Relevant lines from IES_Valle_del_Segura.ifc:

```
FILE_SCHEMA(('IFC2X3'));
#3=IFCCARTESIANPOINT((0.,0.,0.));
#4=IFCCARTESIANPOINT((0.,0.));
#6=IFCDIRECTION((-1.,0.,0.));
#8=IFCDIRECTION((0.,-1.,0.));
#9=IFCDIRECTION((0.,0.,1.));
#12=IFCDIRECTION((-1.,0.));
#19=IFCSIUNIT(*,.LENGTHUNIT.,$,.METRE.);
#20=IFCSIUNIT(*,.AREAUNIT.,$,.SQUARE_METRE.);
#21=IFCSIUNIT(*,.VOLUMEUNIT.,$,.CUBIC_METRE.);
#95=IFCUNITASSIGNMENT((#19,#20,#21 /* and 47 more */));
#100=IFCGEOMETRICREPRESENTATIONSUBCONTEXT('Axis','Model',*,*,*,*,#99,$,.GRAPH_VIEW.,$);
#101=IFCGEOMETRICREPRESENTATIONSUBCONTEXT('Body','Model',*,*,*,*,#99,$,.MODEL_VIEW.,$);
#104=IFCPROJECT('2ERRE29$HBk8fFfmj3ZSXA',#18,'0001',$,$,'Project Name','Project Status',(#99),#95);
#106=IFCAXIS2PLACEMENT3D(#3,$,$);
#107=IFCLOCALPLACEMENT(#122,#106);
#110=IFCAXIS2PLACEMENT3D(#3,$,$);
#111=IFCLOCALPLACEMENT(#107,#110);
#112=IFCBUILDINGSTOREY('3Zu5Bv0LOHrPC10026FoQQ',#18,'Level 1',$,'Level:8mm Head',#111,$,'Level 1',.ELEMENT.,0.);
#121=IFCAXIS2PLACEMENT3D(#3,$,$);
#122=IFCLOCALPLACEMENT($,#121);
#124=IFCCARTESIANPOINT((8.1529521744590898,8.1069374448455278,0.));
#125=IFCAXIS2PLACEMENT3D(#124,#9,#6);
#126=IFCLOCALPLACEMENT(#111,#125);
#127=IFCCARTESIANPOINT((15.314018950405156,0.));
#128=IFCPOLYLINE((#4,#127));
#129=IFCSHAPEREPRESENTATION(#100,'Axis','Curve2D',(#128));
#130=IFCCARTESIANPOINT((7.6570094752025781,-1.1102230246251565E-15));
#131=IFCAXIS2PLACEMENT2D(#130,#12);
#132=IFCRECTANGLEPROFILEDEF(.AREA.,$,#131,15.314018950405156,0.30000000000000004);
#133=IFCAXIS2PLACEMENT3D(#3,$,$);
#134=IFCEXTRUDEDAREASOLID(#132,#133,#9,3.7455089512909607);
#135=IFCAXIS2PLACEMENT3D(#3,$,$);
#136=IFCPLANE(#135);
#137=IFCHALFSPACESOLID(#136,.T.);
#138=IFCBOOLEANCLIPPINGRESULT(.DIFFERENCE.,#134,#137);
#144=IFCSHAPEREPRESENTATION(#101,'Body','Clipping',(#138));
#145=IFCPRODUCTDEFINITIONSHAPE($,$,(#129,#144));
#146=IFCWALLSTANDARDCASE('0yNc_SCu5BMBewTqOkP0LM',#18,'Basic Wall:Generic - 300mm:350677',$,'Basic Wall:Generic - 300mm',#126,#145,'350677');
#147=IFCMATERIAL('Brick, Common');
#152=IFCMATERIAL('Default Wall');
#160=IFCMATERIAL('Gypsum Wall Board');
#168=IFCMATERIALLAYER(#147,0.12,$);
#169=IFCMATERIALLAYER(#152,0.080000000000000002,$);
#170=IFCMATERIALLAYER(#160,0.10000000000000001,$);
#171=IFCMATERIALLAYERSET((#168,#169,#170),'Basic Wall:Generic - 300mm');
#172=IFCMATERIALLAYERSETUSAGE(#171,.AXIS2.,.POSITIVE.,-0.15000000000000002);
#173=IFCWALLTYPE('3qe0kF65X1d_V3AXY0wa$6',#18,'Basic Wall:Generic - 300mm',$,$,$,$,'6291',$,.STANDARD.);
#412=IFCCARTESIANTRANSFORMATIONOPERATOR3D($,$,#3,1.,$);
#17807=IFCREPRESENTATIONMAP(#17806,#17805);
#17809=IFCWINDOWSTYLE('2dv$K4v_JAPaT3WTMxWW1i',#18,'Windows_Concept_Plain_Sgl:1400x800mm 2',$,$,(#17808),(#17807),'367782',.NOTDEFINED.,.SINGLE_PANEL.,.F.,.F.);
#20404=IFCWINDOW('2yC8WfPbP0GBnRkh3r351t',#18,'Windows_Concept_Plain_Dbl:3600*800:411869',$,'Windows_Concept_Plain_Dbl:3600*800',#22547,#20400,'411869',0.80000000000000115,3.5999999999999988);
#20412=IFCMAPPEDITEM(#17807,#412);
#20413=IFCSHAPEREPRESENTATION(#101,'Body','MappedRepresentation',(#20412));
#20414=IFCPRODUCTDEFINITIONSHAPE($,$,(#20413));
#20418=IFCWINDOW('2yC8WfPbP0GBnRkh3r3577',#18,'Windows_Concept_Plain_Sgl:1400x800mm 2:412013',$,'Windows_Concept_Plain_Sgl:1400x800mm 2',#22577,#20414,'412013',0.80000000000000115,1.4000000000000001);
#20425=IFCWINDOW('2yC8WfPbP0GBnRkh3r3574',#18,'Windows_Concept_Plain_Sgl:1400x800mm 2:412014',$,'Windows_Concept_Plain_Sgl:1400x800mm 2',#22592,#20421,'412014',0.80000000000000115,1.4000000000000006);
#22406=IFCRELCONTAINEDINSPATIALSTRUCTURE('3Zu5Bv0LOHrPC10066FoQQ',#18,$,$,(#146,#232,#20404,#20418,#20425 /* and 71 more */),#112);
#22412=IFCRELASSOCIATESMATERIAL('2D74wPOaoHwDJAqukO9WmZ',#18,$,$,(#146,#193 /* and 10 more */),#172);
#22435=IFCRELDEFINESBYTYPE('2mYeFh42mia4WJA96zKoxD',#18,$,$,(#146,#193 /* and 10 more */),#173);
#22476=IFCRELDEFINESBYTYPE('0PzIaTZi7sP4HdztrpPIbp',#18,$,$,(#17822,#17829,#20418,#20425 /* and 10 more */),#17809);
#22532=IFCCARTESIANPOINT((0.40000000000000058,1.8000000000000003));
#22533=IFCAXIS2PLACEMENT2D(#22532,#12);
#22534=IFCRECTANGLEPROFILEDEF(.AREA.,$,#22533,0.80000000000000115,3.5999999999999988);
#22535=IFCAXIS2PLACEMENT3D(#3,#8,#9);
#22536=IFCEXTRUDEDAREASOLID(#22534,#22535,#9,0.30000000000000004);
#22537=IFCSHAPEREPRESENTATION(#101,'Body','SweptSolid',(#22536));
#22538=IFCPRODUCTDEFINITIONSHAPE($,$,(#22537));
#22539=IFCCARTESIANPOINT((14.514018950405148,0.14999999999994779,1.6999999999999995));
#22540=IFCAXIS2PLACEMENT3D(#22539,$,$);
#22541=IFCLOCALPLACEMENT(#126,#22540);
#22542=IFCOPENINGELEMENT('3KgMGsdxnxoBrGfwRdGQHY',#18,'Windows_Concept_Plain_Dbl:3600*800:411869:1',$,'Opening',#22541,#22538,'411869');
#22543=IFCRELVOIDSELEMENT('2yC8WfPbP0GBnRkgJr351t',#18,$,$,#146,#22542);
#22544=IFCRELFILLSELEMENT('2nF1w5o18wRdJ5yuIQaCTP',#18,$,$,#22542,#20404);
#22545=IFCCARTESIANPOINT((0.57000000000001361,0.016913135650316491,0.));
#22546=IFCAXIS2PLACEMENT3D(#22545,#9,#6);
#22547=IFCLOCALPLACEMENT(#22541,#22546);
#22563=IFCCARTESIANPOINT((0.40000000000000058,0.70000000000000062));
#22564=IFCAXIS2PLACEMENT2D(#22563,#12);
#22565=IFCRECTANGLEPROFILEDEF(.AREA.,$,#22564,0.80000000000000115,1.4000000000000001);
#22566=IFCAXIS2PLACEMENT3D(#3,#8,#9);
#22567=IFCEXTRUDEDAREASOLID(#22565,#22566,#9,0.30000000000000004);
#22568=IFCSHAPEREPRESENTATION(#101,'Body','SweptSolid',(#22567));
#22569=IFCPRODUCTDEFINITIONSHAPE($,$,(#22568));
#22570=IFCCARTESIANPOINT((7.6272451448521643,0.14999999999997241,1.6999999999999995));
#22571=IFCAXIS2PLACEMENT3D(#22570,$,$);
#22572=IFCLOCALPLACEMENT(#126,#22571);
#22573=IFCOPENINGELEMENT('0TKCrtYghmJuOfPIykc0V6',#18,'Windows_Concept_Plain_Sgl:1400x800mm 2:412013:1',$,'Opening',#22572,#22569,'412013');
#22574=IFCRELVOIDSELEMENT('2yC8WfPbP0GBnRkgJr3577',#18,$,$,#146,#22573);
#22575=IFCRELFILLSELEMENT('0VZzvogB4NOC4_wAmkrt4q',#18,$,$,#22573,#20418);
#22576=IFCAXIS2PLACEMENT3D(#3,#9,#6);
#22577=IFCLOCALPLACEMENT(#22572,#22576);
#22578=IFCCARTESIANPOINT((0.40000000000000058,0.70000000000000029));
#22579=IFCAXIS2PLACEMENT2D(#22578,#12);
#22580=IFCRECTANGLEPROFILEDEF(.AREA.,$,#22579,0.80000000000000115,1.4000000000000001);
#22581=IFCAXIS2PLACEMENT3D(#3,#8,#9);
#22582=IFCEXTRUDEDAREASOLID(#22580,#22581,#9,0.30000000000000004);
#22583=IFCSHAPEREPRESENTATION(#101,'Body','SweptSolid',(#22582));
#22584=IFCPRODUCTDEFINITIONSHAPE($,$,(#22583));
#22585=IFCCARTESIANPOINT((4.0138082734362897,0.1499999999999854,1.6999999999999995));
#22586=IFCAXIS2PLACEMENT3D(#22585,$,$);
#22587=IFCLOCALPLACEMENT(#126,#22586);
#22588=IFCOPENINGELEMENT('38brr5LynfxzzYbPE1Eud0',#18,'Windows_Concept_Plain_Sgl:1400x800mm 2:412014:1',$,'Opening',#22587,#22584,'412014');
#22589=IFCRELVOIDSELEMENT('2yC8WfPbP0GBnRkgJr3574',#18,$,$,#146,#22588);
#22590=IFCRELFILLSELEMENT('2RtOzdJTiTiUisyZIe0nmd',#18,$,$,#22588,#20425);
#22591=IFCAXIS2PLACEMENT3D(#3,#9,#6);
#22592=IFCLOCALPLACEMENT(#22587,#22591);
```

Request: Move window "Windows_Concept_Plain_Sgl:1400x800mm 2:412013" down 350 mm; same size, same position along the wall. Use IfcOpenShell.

```python
import numpy as np
import ifcopenshell
import ifcopenshell.api.geometry
import ifcopenshell.util.placement
import ifcopenshell.util.unit

model = ifcopenshell.open("IES_Valle_del_Segura.ifc")
unit_scale = ifcopenshell.util.unit.calculate_unit_scale(model)

window = model.by_guid("2yC8WfPbP0GBnRkh3r3577")
opening = window.FillsVoids[0].RelatingOpeningElement
dz = -0.35 / unit_scale

shift = np.array([0.0, 0.0, dz])
# The window is placed relative to its opening, so it follows when the opening moves.
matrix = ifcopenshell.util.placement.get_local_placement(opening.ObjectPlacement)
matrix[:3, 3] += shift
ifcopenshell.api.geometry.edit_object_placement(
    model, product=opening, matrix=matrix, is_si=False, should_transform_children=True
)

print(f"moved by {dz * unit_scale:+.3f} m")

model.write("IES_Valle_del_Segura_edited.ifc")
```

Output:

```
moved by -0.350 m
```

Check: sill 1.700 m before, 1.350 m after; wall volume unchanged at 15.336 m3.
